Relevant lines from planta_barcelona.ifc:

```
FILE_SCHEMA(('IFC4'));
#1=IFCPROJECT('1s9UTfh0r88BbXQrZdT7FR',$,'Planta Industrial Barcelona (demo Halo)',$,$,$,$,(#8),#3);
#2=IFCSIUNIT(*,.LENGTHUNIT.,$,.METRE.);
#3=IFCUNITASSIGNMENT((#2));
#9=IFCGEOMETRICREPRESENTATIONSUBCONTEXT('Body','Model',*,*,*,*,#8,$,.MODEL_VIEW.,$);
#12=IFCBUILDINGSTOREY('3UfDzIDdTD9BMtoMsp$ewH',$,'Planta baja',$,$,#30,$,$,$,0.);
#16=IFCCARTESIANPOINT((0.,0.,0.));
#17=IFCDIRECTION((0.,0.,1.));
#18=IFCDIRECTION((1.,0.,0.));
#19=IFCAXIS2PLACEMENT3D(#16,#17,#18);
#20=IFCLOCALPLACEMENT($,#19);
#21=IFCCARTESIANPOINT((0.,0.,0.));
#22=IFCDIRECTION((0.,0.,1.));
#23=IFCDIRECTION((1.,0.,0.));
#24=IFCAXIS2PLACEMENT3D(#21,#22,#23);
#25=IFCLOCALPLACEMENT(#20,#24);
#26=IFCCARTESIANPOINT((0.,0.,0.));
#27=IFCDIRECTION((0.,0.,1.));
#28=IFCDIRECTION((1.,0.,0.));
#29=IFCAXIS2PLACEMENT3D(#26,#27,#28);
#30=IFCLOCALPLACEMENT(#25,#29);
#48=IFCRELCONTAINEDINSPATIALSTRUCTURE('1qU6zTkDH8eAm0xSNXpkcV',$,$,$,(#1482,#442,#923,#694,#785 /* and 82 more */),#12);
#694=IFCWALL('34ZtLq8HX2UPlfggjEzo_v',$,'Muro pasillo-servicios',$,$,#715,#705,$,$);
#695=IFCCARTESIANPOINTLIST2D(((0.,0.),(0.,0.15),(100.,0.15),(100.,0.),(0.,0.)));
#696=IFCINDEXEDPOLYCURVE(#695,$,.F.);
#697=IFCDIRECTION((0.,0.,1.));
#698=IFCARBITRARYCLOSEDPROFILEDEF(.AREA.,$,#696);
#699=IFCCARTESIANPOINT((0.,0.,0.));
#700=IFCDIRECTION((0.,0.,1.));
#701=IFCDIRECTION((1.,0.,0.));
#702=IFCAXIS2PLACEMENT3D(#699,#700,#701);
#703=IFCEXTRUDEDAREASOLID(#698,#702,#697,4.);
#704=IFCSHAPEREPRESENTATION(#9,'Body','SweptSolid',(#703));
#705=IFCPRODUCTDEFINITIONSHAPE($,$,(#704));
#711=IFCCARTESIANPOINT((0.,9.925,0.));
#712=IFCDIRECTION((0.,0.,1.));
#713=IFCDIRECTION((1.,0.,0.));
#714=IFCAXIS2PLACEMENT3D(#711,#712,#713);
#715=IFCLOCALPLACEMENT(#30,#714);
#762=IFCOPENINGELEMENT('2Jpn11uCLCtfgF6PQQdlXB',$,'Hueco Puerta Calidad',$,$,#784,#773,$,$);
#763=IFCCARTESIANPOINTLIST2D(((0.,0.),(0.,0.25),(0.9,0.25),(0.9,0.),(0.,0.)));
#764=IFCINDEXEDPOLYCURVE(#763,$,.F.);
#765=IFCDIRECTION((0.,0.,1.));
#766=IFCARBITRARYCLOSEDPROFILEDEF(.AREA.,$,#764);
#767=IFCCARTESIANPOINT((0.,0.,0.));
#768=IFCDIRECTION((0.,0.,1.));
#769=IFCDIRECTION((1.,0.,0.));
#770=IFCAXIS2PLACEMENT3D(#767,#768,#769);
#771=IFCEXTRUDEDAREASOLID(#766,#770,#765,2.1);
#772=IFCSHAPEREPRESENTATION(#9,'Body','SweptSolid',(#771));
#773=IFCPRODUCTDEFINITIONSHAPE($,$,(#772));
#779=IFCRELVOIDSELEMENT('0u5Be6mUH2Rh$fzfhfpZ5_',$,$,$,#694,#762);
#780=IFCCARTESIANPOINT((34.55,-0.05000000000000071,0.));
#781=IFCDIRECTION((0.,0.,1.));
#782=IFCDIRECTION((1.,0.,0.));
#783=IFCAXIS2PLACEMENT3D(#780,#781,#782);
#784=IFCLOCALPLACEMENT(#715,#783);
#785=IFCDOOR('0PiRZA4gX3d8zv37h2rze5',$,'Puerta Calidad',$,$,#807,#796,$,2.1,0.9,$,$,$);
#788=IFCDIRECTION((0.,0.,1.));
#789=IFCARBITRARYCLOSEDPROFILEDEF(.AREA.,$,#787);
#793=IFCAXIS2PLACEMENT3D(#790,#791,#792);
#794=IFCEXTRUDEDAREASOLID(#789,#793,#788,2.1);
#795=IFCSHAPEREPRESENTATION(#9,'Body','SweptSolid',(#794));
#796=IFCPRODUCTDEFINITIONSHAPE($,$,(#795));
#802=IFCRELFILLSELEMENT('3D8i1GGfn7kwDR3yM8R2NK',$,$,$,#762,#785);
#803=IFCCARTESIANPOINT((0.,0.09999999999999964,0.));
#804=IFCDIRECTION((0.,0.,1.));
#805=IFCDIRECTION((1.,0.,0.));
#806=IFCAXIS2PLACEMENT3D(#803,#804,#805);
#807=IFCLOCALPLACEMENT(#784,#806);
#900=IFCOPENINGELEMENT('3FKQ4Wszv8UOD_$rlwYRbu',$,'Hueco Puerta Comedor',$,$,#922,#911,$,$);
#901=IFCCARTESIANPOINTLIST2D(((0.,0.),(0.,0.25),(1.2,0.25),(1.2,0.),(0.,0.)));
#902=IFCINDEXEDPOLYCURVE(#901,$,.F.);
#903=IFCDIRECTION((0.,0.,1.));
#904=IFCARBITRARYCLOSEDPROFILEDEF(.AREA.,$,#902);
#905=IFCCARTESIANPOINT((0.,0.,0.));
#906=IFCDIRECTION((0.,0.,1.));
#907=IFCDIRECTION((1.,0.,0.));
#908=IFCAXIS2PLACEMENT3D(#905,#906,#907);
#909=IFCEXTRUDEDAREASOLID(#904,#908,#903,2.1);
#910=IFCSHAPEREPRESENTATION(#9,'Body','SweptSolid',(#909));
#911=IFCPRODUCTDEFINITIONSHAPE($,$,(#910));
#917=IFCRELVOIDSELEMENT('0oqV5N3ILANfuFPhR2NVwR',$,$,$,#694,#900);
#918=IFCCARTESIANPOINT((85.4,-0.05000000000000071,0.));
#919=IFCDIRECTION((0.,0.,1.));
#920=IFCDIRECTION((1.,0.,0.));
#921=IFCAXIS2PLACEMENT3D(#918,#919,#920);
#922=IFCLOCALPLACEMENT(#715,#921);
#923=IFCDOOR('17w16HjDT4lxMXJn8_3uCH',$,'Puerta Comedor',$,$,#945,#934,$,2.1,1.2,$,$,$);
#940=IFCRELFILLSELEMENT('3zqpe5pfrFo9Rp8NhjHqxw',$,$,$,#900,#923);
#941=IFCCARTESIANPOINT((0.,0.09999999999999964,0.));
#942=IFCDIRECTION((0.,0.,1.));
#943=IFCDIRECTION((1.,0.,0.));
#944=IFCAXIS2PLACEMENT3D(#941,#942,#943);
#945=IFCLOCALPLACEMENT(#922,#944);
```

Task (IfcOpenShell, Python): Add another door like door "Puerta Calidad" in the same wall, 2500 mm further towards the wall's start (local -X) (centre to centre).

```python
import ifcopenshell
import ifcopenshell.api.feature
import ifcopenshell.api.geometry
import ifcopenshell.api.root
import ifcopenshell.geom
import ifcopenshell.util.element
import ifcopenshell.util.placement
import ifcopenshell.util.shape

model = ifcopenshell.open("planta_barcelona.ifc")
settings = ifcopenshell.geom.settings()


def volume(element):
    """Net volume in cubic metres, openings subtracted."""
    shape = ifcopenshell.geom.create_shape(settings, element)
    return ifcopenshell.util.shape.get_volume(shape.geometry)


door = model.by_id(785)
opening = door.FillsVoids[0].RelatingOpeningElement
wall = opening.VoidsElements[0].RelatingBuildingElement
before = volume(wall)
shift = ifcopenshell.util.placement.get_local_placement(wall.ObjectPlacement)[:3, 0] * -2.5

# copy_class copies the void relationship, type, container and properties, but no geometry.
new_opening = ifcopenshell.api.root.copy_class(model, product=opening)
new_opening.Representation = ifcopenshell.util.element.copy_deep(
    model, opening.Representation, exclude=["IfcGeometricRepresentationContext", "IfcRepresentationMap"]
)
new_door = ifcopenshell.api.root.copy_class(model, product=door)
new_door.Representation = ifcopenshell.util.element.copy_deep(
    model, door.Representation, exclude=["IfcGeometricRepresentationContext", "IfcRepresentationMap"]
)
ifcopenshell.api.feature.add_filling(model, opening=new_opening, element=new_door)

for old, new in ((opening, new_opening), (door, new_door)):
    matrix = ifcopenshell.util.placement.get_local_placement(old.ObjectPlacement)
    matrix[:3, 3] += shift
    ifcopenshell.api.geometry.edit_object_placement(model, product=new, matrix=matrix, is_si=False)

after = volume(wall)

print(f"wall volume {before:.3f} -> {after:.3f} m3")

model.write("planta_barcelona-out.ifc")
```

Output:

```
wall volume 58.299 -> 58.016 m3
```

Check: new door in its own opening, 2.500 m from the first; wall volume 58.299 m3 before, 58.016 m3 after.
